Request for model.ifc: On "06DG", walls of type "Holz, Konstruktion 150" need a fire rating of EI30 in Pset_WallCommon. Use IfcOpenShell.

First a look at what the model holds.

```python
import ifcopenshell
import ifcopenshell.util.element

model = ifcopenshell.open("model.ifc")
print(model.schema)
storey = next(s for s in model.by_type("IfcBuildingStorey") if s.Name == "06DG")
walls = [e for e in ifcopenshell.util.element.get_decomposition(storey) if e.is_a("IfcWall")]
seen = {}
for e in walls:
    element_type = ifcopenshell.util.element.get_type(e)
    key = (element_type.Name if element_type != e and element_type else None, ifcopenshell.util.element.get_pset(e, "Pset_WallCommon", "FireRating"))
    seen[key] = seen.get(key, 0) + 1
for (name, value), count in sorted(seen.items(), key=str):
    print(count, "x", name, "|", value)
```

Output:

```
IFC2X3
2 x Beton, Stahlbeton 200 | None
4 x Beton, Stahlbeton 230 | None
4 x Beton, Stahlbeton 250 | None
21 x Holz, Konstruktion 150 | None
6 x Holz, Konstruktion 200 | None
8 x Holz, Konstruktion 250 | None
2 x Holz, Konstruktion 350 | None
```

```python
import ifcopenshell
import ifcopenshell.api.pset
import ifcopenshell.util.element

model = ifcopenshell.open("model.ifc")

storey = next(s for s in model.by_type("IfcBuildingStorey") if s.Name == "06DG")
walls = [e for e in ifcopenshell.util.element.get_decomposition(storey) if e.is_a("IfcWall")]

count = 0
for e in walls:
    element_type = ifcopenshell.util.element.get_type(e)
    if element_type in (None, e) or element_type.Name != "Holz, Konstruktion 150":
        continue
    found = ifcopenshell.util.element.get_pset(e, "Pset_WallCommon", should_inherit=False)
    if found:
        pset = model.by_id(found["id"])
        if len(ifcopenshell.util.element.get_elements_by_pset(pset)) > 1:
            pset = ifcopenshell.api.pset.unshare_pset(model, products=[e], pset=pset)[0]
    else:
        pset = ifcopenshell.api.pset.add_pset(model, product=e, name="Pset_WallCommon")
    ifcopenshell.api.pset.edit_pset(model, pset=pset, properties={"FireRating": "EI30"})
    count += 1

print(count, "walls updated")

model.write("model_rev.ifc")
```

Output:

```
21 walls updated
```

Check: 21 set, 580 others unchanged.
